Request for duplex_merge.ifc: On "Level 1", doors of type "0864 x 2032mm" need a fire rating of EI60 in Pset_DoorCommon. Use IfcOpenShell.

First a look at what the model holds.

```python
import ifcopenshell
import ifcopenshell.util.element

model = ifcopenshell.open("duplex_merge.ifc")
print(model.schema)
storey = next(s for s in model.by_type("IfcBuildingStorey") if s.Name == "Level 1")
doors = [e for e in ifcopenshell.util.element.get_decomposition(storey) if e.is_a("IfcDoor")]
seen = {}
for e in doors:
    element_type = ifcopenshell.util.element.get_type(e)
    key = (element_type.Name if element_type != e and element_type else None, ifcopenshell.util.element.get_pset(e, "Pset_DoorCommon", "FireRating"))
    seen[key] = seen.get(key, 0) + 1
for (name, value), count in sorted(seen.items(), key=str):
    print(count, "x", name, "|", value)
```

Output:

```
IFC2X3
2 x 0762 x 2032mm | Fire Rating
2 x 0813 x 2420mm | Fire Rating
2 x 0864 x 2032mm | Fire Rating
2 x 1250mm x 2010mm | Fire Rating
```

```python
import ifcopenshell
import ifcopenshell.api.pset
import ifcopenshell.util.element

model = ifcopenshell.open("duplex_merge.ifc")

storey = next(s for s in model.by_type("IfcBuildingStorey") if s.Name == "Level 1")
doors = [e for e in ifcopenshell.util.element.get_decomposition(storey) if e.is_a("IfcDoor")]

count = 0
for e in doors:
    element_type = ifcopenshell.util.element.get_type(e)
    if element_type in (None, e) or element_type.Name != "0864 x 2032mm":
        continue
    # add_pset returns the element's existing set when there is one.
    pset = ifcopenshell.api.pset.add_pset(model, product=e, name="Pset_DoorCommon")
    ifcopenshell.api.pset.edit_pset(model, pset=pset, properties={"FireRating": "EI60"})
    count += 1

print(count, "doors updated")

model.write("duplex_merge-out.ifc")
```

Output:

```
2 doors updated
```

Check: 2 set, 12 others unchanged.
